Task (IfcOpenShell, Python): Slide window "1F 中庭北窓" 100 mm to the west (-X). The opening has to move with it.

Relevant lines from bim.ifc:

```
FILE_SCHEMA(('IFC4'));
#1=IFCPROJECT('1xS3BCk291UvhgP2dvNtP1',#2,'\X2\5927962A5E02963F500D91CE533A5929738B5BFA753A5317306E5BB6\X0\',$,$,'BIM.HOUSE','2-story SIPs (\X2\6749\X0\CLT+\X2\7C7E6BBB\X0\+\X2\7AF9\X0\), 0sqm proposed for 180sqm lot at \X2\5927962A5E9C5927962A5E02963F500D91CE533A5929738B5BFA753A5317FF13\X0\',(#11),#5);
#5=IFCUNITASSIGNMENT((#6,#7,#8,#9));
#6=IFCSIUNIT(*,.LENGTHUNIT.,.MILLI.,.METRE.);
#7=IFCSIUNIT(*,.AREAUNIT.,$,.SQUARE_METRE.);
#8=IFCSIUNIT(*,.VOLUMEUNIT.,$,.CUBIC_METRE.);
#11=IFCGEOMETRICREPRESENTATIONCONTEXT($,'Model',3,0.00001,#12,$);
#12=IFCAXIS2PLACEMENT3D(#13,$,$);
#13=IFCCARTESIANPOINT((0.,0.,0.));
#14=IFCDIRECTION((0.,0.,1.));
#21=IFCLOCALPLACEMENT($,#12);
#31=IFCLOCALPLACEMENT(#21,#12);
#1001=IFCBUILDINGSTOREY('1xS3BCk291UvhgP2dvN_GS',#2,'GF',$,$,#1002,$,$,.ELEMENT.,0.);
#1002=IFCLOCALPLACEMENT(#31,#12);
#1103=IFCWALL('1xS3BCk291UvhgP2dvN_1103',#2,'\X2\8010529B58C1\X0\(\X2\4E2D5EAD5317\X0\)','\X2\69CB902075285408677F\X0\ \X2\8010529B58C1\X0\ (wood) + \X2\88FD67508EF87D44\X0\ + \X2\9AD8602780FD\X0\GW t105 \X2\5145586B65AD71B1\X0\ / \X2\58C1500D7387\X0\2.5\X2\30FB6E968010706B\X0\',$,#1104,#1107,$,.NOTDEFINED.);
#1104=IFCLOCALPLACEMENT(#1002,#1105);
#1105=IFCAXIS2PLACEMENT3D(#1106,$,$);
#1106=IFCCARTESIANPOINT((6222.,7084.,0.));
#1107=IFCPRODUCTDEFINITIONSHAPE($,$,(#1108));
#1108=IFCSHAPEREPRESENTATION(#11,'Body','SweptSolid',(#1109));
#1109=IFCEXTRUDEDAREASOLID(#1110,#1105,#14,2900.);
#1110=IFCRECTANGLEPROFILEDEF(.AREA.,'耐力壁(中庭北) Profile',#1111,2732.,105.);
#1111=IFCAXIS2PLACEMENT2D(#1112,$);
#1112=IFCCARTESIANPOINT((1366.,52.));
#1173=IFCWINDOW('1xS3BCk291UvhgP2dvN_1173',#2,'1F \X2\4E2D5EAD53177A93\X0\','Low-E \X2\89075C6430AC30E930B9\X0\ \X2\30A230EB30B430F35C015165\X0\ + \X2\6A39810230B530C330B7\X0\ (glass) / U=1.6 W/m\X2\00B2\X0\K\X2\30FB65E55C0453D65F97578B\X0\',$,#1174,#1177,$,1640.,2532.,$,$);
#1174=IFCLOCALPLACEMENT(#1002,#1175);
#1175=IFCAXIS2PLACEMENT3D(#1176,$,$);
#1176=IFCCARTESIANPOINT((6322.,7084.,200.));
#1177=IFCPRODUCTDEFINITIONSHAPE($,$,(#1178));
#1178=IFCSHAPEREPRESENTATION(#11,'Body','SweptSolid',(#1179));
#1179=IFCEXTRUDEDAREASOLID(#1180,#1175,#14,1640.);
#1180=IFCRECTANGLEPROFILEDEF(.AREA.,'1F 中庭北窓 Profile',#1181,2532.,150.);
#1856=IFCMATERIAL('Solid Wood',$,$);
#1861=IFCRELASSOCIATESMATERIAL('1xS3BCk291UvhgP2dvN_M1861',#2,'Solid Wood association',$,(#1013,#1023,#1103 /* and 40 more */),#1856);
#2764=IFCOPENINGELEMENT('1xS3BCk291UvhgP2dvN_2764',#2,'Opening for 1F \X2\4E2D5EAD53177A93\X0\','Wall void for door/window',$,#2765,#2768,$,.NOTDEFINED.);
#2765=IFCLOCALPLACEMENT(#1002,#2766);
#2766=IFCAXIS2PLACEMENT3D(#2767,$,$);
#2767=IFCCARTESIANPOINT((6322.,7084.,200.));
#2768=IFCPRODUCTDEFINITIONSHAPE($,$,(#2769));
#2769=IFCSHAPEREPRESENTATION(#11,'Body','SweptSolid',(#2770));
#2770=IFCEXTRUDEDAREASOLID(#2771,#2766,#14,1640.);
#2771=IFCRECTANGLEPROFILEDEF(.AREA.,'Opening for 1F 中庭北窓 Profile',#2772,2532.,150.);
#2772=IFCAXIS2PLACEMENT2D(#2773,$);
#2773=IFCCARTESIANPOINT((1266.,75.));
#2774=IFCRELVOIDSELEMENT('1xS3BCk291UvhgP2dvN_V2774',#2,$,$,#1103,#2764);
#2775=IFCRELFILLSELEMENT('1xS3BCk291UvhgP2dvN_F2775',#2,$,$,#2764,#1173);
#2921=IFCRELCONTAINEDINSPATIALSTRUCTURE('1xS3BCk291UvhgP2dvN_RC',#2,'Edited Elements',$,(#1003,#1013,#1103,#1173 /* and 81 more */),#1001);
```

```python
import ifcopenshell
import ifcopenshell.api.geometry
import ifcopenshell.util.placement
import ifcopenshell.util.unit

model = ifcopenshell.open("bim.ifc")
unit_scale = ifcopenshell.util.unit.calculate_unit_scale(model)

window = model.by_id(1173)
opening = window.FillsVoids[0].RelatingOpeningElement
wall = opening.VoidsElements[0].RelatingBuildingElement

wall_matrix = ifcopenshell.util.placement.get_local_placement(wall.ObjectPlacement)
shift = wall_matrix[:3, 0] * -0.1 / unit_scale
before = ifcopenshell.util.placement.get_local_placement(window.ObjectPlacement)[:3, 3].copy()

# The window is not placed relative to its opening, so move both.
for product in (opening, window):
    matrix = ifcopenshell.util.placement.get_local_placement(product.ObjectPlacement)
    matrix[:3, 3] += shift
    ifcopenshell.api.geometry.edit_object_placement(model, product=product, matrix=matrix, is_si=False)

after = ifcopenshell.util.placement.get_local_placement(window.ObjectPlacement)[:3, 3]
print("window moved by", (after - before).round(3) + 0.0)

model.write("bim_v2.ifc")
```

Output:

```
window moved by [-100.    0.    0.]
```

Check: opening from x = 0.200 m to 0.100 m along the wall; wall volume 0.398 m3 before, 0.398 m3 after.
